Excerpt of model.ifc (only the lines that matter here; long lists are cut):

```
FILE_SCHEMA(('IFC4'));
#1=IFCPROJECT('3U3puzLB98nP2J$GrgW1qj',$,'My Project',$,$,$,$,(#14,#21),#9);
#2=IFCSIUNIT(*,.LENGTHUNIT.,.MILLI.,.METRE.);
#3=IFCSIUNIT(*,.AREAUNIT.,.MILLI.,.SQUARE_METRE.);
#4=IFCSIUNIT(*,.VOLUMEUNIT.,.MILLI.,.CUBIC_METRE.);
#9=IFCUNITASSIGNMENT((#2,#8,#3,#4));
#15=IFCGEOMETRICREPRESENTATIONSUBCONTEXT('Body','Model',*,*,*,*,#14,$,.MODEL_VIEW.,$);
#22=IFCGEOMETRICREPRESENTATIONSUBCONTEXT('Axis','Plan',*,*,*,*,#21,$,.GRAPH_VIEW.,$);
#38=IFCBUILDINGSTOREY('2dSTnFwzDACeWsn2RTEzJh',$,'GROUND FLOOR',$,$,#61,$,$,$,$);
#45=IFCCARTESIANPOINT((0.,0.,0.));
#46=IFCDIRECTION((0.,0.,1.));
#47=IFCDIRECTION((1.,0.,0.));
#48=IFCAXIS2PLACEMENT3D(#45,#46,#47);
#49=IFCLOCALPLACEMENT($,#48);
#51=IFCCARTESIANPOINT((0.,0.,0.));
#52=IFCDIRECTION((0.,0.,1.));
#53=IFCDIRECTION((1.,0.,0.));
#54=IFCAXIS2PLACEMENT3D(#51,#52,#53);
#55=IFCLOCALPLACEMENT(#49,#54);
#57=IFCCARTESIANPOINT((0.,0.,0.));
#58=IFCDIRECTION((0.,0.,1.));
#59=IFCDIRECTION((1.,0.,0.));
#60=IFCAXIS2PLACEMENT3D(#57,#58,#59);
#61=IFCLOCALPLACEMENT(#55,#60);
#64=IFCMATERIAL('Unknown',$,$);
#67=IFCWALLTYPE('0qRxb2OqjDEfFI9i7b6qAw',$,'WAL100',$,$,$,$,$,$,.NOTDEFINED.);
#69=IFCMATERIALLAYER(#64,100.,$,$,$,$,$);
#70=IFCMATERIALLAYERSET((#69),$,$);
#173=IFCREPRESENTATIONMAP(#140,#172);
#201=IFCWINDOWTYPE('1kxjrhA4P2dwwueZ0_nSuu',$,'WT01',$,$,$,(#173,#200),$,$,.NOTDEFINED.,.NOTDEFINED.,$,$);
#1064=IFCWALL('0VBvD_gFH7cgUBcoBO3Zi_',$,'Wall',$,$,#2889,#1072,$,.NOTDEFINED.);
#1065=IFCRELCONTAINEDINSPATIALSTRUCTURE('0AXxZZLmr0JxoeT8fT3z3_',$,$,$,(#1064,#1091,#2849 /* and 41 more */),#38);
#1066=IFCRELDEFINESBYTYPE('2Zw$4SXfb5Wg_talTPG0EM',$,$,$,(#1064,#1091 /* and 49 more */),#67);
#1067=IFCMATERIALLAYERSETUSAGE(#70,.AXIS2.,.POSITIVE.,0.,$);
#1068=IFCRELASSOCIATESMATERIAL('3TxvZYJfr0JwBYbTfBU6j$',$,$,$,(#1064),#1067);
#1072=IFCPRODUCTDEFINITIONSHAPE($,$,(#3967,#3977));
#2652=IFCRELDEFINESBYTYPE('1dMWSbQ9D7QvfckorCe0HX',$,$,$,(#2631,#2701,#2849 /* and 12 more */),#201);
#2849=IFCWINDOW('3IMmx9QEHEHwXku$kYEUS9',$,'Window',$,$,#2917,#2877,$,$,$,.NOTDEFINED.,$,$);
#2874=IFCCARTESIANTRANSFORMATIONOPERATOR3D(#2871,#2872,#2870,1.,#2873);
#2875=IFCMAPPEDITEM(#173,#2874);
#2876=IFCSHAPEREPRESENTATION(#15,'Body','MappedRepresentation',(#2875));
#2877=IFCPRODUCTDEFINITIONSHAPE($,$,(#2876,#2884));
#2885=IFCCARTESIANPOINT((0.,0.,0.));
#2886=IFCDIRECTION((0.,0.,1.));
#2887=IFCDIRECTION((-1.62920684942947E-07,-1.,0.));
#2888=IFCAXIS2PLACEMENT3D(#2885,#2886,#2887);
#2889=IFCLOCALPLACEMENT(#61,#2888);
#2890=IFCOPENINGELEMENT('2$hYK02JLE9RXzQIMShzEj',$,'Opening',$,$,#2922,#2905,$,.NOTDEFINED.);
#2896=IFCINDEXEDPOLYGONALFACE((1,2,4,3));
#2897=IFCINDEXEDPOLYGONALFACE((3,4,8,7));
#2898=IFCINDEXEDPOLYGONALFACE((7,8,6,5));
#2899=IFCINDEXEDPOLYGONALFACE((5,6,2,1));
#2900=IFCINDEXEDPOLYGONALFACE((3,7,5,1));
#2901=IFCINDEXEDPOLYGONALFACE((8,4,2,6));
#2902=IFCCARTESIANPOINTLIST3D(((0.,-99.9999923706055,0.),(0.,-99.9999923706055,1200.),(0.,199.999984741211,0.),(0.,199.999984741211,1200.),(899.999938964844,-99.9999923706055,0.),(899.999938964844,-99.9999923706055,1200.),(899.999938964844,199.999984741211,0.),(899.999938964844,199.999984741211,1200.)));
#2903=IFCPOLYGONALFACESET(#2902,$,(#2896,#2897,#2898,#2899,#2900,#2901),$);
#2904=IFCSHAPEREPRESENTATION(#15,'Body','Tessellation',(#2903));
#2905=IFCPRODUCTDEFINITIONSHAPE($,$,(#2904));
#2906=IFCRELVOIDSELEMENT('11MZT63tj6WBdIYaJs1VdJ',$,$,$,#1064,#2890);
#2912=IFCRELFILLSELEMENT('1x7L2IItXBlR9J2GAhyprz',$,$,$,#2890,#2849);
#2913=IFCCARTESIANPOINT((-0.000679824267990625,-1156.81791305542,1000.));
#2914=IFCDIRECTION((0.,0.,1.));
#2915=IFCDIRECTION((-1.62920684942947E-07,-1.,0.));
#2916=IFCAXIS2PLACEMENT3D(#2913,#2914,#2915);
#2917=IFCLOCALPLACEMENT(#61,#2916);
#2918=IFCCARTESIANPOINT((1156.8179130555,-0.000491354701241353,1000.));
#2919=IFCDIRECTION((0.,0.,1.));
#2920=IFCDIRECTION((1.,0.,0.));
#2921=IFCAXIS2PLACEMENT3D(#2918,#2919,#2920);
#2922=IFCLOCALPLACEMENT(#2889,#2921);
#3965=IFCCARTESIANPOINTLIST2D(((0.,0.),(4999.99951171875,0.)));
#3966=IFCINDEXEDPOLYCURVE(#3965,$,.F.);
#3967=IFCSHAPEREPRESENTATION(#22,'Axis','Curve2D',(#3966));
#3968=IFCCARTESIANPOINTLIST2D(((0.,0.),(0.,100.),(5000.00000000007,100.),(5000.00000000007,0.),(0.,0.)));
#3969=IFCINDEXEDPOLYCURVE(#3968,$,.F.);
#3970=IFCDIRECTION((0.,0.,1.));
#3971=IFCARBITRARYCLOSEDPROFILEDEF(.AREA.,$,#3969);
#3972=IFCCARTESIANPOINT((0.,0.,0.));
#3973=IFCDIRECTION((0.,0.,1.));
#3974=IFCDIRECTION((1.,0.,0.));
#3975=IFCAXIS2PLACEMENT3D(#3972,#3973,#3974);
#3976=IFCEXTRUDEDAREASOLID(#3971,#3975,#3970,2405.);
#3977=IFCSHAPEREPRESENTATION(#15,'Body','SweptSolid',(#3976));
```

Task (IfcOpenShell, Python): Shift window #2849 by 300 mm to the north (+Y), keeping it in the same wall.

```python
import ifcopenshell
import ifcopenshell.api.geometry
import ifcopenshell.util.placement
import ifcopenshell.util.unit

model = ifcopenshell.open("model.ifc")
unit_scale = ifcopenshell.util.unit.calculate_unit_scale(model)

window = model.by_guid("3IMmx9QEHEHwXku$kYEUS9")
opening = window.FillsVoids[0].RelatingOpeningElement
wall = opening.VoidsElements[0].RelatingBuildingElement

wall_matrix = ifcopenshell.util.placement.get_local_placement(wall.ObjectPlacement)
shift = wall_matrix[:3, 0] * -0.3 / unit_scale
before = ifcopenshell.util.placement.get_local_placement(window.ObjectPlacement)[:3, 3].copy()

# The window is not placed relative to its opening, so move both.
for product in (opening, window):
    matrix = ifcopenshell.util.placement.get_local_placement(product.ObjectPlacement)
    matrix[:3, 3] += shift
    ifcopenshell.api.geometry.edit_object_placement(model, product=product, matrix=matrix, is_si=False)

after = ifcopenshell.util.placement.get_local_placement(window.ObjectPlacement)[:3, 3]
print("window moved by", (after - before).round(3) + 0.0)

model.write("model-out.ifc")
```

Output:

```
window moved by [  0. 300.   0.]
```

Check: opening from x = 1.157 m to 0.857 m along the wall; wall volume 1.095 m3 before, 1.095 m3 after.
